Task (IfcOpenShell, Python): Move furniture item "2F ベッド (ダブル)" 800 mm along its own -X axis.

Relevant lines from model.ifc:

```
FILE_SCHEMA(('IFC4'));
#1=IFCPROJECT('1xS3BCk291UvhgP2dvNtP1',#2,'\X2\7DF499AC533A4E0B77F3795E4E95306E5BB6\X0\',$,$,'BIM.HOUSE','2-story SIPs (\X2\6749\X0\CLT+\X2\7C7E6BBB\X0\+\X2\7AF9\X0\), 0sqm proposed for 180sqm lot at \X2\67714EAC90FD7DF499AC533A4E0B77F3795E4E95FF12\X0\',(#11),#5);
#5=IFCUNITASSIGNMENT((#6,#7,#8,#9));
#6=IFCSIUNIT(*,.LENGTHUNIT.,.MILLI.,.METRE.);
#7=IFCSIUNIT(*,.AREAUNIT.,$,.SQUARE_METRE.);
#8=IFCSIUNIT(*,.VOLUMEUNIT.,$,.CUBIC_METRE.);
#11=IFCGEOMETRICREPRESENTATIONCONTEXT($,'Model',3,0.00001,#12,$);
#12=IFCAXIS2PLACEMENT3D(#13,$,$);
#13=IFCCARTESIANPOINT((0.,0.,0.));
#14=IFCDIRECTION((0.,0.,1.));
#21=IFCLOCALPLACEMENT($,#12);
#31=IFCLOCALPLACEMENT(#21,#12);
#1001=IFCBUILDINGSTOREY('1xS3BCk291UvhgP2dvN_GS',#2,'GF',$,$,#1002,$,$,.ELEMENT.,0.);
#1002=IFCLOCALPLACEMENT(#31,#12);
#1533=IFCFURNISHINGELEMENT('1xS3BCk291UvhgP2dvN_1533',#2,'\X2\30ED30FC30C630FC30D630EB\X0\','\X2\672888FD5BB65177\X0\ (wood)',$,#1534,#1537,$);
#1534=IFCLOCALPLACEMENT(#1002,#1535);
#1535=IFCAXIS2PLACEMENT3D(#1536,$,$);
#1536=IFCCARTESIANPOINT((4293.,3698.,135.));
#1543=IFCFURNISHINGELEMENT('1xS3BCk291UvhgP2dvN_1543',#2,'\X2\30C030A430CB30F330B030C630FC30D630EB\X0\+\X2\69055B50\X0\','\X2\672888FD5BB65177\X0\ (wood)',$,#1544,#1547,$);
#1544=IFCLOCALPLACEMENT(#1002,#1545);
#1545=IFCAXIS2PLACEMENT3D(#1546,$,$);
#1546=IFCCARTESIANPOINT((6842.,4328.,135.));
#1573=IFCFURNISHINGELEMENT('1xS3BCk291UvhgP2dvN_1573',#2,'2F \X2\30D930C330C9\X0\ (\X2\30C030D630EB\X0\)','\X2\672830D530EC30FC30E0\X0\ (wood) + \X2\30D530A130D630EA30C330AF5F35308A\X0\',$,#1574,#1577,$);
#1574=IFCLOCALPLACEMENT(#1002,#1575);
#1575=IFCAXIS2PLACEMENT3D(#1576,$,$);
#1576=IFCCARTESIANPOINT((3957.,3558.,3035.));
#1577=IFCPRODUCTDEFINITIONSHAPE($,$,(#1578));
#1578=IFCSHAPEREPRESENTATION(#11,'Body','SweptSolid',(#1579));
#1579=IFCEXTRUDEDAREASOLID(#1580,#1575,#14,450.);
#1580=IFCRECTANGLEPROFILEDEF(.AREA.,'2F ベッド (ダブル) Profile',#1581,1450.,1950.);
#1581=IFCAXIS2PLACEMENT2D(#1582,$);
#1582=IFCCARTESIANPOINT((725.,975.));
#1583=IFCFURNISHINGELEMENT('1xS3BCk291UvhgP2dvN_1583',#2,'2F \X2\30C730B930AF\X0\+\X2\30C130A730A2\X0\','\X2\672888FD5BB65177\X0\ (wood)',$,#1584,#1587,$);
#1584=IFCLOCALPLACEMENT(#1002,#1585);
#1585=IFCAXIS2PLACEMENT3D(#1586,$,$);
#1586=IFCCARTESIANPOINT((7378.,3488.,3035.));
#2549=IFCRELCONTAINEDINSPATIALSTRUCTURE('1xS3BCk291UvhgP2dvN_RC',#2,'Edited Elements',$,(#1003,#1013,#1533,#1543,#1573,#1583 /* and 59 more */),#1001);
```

```python
import ifcopenshell
import ifcopenshell.api.geometry
import ifcopenshell.util.placement
import ifcopenshell.util.unit

model = ifcopenshell.open("model.ifc")
unit_scale = ifcopenshell.util.unit.calculate_unit_scale(model)

item = model.by_id(1573)
matrix = ifcopenshell.util.placement.get_local_placement(item.ObjectPlacement)
matrix[:3, 3] -= matrix[:3, 0] * 0.8 / unit_scale
ifcopenshell.api.geometry.edit_object_placement(model, product=item, matrix=matrix, is_si=False)

print(ifcopenshell.util.placement.get_local_placement(item.ObjectPlacement).round(3) + 0.0)

model.write("model_updated.ifc")
```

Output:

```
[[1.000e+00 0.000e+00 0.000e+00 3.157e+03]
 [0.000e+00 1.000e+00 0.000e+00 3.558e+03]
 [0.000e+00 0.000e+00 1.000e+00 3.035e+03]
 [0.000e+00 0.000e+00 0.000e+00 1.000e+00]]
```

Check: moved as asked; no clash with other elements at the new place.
